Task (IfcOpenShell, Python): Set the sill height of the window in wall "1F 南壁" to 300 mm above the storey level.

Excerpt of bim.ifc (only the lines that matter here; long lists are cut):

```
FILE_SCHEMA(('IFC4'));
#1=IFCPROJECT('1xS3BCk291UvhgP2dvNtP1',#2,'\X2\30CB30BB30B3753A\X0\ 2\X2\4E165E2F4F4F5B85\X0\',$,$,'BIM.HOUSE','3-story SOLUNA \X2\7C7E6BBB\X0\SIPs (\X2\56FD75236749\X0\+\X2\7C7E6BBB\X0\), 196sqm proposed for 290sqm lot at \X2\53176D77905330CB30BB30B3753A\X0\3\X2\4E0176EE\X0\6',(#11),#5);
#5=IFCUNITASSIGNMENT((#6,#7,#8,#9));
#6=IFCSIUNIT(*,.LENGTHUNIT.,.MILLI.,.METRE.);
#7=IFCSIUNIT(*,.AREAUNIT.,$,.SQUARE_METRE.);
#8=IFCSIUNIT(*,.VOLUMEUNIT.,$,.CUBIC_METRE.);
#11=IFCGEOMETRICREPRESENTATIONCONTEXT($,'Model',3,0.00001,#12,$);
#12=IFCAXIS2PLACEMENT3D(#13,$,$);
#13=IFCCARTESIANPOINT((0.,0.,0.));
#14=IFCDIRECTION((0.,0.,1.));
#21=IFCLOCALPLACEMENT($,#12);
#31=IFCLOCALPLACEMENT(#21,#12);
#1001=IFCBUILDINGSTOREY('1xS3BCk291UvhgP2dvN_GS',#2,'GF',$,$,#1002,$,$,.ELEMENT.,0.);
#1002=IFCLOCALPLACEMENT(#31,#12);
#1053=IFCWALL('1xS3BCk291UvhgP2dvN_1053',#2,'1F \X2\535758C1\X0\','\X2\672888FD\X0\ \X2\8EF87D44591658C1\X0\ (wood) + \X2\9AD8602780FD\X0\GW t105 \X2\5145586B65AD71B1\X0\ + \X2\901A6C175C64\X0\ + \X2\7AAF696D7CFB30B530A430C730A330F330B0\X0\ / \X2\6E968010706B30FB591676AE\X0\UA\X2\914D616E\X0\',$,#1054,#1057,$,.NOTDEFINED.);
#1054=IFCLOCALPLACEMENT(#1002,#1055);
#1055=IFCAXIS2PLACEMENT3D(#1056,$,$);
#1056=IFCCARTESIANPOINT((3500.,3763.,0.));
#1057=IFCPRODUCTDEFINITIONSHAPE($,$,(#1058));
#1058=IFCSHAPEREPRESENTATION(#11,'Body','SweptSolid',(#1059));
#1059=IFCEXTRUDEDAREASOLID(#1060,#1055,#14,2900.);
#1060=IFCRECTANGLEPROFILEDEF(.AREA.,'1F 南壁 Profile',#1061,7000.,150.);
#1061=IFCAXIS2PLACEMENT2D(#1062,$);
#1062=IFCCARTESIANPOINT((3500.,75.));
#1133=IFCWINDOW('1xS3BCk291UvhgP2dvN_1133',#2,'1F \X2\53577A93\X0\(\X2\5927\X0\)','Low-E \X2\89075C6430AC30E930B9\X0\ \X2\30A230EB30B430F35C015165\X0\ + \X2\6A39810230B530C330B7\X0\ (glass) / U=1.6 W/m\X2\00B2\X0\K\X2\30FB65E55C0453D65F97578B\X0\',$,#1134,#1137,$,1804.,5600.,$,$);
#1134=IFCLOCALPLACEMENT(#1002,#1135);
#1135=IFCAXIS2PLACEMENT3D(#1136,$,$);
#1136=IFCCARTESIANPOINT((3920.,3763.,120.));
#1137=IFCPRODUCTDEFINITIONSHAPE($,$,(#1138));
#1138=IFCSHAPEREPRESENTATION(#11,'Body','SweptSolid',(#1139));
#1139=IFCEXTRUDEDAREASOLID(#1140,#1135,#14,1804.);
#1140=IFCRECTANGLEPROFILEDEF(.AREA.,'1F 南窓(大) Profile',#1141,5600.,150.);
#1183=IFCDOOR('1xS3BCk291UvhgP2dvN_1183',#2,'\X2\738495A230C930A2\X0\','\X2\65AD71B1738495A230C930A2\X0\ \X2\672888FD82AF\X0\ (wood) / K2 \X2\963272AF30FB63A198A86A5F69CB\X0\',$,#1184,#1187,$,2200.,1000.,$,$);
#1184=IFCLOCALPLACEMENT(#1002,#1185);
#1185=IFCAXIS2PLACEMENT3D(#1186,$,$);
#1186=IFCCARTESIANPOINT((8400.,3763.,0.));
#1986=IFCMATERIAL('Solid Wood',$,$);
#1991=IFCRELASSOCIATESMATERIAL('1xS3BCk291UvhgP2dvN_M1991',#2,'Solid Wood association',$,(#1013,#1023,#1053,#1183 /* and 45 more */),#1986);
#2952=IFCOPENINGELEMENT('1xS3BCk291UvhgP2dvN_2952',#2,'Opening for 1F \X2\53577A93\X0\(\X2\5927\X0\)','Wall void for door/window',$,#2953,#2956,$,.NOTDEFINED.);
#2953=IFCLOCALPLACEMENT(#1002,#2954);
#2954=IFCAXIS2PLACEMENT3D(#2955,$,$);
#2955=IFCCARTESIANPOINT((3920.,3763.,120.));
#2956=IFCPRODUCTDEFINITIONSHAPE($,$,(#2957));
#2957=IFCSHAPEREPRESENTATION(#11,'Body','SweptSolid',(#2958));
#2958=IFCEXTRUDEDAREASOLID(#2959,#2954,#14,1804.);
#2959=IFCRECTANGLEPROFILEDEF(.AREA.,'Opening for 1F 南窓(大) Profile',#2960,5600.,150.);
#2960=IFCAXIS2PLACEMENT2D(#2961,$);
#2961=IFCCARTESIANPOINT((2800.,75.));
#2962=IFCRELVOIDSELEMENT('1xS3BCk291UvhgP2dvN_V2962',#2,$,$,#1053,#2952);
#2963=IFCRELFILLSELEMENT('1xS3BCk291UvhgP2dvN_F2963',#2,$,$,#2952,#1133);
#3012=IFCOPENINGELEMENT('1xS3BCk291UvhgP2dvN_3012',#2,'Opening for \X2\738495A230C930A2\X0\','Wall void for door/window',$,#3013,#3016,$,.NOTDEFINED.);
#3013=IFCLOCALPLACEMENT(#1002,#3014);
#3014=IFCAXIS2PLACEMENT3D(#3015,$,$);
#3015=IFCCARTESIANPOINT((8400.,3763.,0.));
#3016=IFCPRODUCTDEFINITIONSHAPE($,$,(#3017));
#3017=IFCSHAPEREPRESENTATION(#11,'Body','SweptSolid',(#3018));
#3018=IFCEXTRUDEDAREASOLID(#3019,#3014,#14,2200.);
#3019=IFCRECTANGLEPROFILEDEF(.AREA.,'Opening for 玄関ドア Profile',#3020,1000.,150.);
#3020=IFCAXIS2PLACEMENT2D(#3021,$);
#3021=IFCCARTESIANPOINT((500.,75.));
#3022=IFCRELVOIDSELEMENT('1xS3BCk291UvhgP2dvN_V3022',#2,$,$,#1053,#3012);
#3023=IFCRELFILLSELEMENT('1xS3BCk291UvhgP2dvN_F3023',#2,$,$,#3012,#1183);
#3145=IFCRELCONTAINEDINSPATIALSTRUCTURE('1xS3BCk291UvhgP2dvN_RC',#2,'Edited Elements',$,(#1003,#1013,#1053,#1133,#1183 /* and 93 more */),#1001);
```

```python
import numpy as np
import ifcopenshell
import ifcopenshell.api.geometry
import ifcopenshell.geom
import ifcopenshell.util.element
import ifcopenshell.util.placement
import ifcopenshell.util.shape
import ifcopenshell.util.unit

model = ifcopenshell.open("bim.ifc")
unit_scale = ifcopenshell.util.unit.calculate_unit_scale(model)

window = model.by_guid("1xS3BCk291UvhgP2dvN_1133")
opening = window.FillsVoids[0].RelatingOpeningElement
storey = ifcopenshell.util.element.get_container(window, ifc_class="IfcBuildingStorey")
level = ifcopenshell.util.placement.get_local_placement(storey.ObjectPlacement)[2, 3]

# The opening's origin need not be at the sill, so measure its lowest point.
shape = ifcopenshell.geom.create_shape(ifcopenshell.geom.settings(), opening)
bottom = ifcopenshell.util.shape.get_shape_bottom_elevation(shape, shape.geometry) / unit_scale
dz = level + 300.0 - bottom

shift = np.array([0.0, 0.0, dz])
# The window is not placed relative to its opening, so move both.
for product in (opening, window):
    matrix = ifcopenshell.util.placement.get_local_placement(product.ObjectPlacement)
    matrix[:3, 3] += shift
    ifcopenshell.api.geometry.edit_object_placement(model, product=product, matrix=matrix, is_si=False)

print(f"moved by {dz * unit_scale:+.3f} m")

model.write("bim_v2.ifc")
```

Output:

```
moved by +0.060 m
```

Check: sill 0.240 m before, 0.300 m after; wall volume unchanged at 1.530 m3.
